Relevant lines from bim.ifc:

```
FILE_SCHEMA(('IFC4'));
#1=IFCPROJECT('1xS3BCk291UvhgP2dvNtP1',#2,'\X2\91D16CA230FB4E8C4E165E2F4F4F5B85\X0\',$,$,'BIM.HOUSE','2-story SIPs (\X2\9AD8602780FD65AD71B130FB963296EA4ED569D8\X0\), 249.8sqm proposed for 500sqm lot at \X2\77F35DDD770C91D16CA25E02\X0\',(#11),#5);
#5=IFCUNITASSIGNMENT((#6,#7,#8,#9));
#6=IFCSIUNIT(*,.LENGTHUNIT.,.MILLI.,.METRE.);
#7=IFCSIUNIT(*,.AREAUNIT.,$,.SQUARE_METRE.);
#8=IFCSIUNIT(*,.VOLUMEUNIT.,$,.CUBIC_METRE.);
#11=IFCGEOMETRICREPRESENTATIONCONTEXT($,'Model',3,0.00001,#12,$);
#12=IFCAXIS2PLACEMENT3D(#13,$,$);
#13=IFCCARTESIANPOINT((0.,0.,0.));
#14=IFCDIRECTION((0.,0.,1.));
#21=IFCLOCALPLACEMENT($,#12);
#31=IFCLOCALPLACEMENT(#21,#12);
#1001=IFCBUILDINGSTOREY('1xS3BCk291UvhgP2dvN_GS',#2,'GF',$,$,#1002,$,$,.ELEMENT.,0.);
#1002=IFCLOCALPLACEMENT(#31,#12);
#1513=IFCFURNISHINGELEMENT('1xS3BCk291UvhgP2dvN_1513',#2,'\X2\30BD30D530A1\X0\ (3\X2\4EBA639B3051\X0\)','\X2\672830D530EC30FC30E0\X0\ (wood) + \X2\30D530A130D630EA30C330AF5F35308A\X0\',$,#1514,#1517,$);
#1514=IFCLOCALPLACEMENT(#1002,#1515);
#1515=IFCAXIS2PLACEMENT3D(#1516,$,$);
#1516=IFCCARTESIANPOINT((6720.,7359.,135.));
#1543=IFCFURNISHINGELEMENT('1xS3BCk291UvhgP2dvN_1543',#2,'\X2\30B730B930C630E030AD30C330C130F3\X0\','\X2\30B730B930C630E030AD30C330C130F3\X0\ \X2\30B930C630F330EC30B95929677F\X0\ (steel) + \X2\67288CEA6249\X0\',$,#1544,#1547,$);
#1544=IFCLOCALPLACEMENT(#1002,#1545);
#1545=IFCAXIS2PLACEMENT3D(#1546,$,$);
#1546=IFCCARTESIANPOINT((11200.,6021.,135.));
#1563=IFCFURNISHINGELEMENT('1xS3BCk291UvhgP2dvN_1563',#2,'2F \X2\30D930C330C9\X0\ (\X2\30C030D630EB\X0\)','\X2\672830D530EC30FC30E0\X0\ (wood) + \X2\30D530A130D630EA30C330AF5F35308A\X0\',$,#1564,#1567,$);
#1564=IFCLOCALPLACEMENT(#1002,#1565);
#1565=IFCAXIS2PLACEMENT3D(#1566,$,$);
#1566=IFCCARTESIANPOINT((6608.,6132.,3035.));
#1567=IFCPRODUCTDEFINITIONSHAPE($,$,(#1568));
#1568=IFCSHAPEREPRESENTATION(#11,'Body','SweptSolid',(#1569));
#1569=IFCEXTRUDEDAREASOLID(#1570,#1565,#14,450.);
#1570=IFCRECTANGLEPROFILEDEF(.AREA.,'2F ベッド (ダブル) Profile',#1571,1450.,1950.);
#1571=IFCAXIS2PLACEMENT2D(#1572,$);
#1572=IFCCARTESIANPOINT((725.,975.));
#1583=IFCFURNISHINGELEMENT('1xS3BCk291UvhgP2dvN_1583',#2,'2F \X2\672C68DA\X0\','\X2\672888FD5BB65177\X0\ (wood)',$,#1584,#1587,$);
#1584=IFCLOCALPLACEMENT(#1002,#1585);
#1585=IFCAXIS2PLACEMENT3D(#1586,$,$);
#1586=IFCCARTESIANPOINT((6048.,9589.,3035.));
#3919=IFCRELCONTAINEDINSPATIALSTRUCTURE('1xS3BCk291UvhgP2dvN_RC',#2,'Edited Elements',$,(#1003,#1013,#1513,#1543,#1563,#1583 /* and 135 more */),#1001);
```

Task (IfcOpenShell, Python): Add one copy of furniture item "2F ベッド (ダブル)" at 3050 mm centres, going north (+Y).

```python
import numpy as np
import ifcopenshell
import ifcopenshell.api.geometry
import ifcopenshell.api.root
import ifcopenshell.util.element
import ifcopenshell.util.placement
import ifcopenshell.util.unit

model = ifcopenshell.open("bim.ifc")
unit_scale = ifcopenshell.util.unit.calculate_unit_scale(model)


def reuse_history(source, copy):
    """copy_class also copies each property set's owner history, people and application; keep the originals."""
    for rel in copy.IsDefinedBy:
        if rel.is_a("IfcRelDefinesByProperties") and (history := rel.RelatingPropertyDefinition.OwnerHistory):
            rel.RelatingPropertyDefinition.OwnerHistory = source.OwnerHistory
            ifcopenshell.util.element.remove_deep2(model, history)


source = model.by_id(1563)
base = ifcopenshell.util.placement.get_local_placement(source.ObjectPlacement)
step = np.array([0.0, 1.0, 0.0]) * 3.05 / unit_scale

for i in range(1, 2):
    copy = ifcopenshell.api.root.copy_class(model, product=source)
    copy.Representation = ifcopenshell.util.element.copy_deep(
        model, source.Representation, exclude=["IfcGeometricRepresentationContext", "IfcRepresentationMap"]
    )
    reuse_history(source, copy)
    matrix = base.copy()
    matrix[:3, 3] += i * step
    print("added at", matrix[:3, 3].round(3) + 0.0)
    ifcopenshell.api.geometry.edit_object_placement(model, product=copy, matrix=matrix, is_si=False)

model.write("bim_updated.ifc")
```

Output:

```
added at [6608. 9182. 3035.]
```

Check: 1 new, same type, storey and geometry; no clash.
